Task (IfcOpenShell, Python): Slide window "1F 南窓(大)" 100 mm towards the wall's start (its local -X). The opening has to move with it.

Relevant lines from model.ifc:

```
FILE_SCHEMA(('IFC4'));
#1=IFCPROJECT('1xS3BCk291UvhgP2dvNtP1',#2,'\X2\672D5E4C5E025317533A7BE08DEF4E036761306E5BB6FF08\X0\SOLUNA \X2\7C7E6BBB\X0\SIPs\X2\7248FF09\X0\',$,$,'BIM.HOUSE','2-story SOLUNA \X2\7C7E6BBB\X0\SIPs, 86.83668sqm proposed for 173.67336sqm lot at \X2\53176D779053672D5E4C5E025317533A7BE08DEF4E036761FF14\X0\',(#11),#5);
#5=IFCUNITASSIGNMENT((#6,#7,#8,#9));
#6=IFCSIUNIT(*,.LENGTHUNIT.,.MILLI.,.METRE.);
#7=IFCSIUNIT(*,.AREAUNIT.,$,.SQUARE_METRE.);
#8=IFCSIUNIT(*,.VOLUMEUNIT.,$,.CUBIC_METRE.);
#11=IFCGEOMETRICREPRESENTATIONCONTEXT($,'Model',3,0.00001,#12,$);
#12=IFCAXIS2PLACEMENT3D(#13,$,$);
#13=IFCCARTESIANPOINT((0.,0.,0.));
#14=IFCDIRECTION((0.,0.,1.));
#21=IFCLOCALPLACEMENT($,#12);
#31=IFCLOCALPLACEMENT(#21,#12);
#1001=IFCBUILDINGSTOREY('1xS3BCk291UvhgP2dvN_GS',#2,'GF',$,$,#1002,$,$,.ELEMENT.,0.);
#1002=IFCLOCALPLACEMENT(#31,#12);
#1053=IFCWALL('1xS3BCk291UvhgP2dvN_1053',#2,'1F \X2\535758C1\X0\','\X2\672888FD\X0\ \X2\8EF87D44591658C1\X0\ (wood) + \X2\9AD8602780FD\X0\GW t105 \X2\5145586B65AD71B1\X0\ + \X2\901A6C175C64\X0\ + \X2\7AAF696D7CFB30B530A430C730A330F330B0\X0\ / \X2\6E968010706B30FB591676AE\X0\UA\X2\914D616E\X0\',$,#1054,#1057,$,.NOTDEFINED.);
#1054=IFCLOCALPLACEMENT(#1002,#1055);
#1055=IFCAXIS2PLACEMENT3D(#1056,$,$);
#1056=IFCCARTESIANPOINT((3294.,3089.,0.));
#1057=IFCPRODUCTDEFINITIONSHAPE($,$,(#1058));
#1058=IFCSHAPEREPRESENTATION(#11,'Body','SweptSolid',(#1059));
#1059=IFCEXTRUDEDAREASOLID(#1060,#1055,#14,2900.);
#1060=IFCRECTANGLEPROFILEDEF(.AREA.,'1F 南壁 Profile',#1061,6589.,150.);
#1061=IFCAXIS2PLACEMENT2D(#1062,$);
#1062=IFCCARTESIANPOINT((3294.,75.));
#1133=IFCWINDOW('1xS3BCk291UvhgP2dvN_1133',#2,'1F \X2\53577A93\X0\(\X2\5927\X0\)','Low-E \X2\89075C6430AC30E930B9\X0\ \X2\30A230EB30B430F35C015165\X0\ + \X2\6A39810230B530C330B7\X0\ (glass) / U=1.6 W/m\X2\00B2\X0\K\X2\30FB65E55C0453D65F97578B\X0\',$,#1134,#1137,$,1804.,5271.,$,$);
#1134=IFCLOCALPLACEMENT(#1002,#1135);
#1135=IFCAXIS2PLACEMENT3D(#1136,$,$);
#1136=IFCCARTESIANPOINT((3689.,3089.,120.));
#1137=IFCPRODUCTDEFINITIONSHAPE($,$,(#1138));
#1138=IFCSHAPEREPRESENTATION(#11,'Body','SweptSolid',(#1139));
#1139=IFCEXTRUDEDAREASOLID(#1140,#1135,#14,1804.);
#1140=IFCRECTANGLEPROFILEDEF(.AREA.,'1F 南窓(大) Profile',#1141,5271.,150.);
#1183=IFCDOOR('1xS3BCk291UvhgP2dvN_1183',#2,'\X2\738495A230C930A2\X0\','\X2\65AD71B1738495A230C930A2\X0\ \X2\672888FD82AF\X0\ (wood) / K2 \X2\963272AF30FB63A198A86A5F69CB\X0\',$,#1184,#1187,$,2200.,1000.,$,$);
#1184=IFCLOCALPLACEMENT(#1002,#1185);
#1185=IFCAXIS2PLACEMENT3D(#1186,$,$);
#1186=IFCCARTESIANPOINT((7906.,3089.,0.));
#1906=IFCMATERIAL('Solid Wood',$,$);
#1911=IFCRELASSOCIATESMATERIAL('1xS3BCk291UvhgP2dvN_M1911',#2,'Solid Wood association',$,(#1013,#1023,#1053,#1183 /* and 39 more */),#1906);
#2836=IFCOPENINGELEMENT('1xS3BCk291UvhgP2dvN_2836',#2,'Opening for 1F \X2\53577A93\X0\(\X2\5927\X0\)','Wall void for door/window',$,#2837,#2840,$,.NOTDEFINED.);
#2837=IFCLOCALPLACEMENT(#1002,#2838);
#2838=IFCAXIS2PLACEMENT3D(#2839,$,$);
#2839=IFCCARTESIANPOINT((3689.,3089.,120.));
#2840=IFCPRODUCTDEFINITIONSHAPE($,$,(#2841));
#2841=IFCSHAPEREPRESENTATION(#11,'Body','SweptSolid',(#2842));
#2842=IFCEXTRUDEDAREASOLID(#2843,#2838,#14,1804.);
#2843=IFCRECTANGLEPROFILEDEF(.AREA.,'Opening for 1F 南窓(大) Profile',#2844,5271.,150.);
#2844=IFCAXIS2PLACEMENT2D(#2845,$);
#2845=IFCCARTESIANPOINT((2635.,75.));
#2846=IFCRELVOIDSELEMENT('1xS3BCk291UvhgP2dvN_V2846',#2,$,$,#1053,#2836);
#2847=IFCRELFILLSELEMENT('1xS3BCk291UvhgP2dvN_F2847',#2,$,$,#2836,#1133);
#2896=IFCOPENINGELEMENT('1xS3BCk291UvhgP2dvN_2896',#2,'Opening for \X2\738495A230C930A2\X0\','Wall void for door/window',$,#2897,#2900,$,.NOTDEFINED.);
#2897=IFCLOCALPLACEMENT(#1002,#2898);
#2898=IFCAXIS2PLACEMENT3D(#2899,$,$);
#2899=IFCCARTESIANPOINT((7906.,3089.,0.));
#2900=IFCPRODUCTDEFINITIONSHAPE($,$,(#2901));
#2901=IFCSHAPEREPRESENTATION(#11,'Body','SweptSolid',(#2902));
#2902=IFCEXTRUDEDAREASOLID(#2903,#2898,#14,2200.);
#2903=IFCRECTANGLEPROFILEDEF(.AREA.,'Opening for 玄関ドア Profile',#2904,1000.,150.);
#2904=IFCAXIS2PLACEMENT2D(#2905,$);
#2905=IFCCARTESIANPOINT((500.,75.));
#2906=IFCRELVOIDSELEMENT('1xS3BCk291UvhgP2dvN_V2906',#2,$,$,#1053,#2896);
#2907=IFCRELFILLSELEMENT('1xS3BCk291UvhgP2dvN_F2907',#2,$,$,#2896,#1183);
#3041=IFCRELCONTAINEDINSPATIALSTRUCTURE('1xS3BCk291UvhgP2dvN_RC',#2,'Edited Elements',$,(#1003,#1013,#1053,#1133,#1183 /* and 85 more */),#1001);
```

```python
import ifcopenshell
import ifcopenshell.api.geometry
import ifcopenshell.util.placement
import ifcopenshell.util.unit

model = ifcopenshell.open("model.ifc")
unit_scale = ifcopenshell.util.unit.calculate_unit_scale(model)

window = model.by_guid("1xS3BCk291UvhgP2dvN_1133")
opening = window.FillsVoids[0].RelatingOpeningElement
wall = opening.VoidsElements[0].RelatingBuildingElement

wall_matrix = ifcopenshell.util.placement.get_local_placement(wall.ObjectPlacement)
shift = wall_matrix[:3, 0] * -0.1 / unit_scale
before = ifcopenshell.util.placement.get_local_placement(window.ObjectPlacement)[:3, 3].copy()

# The window is not placed relative to its opening, so move both.
for product in (opening, window):
    matrix = ifcopenshell.util.placement.get_local_placement(product.ObjectPlacement)
    matrix[:3, 3] += shift
    ifcopenshell.api.geometry.edit_object_placement(model, product=product, matrix=matrix, is_si=False)

after = ifcopenshell.util.placement.get_local_placement(window.ObjectPlacement)[:3, 3]
print("window moved by", (after - before).round(3) + 0.0)

model.write("model_rev.ifc")
```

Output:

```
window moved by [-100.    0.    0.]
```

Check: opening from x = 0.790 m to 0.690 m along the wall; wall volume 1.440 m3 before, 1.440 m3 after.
